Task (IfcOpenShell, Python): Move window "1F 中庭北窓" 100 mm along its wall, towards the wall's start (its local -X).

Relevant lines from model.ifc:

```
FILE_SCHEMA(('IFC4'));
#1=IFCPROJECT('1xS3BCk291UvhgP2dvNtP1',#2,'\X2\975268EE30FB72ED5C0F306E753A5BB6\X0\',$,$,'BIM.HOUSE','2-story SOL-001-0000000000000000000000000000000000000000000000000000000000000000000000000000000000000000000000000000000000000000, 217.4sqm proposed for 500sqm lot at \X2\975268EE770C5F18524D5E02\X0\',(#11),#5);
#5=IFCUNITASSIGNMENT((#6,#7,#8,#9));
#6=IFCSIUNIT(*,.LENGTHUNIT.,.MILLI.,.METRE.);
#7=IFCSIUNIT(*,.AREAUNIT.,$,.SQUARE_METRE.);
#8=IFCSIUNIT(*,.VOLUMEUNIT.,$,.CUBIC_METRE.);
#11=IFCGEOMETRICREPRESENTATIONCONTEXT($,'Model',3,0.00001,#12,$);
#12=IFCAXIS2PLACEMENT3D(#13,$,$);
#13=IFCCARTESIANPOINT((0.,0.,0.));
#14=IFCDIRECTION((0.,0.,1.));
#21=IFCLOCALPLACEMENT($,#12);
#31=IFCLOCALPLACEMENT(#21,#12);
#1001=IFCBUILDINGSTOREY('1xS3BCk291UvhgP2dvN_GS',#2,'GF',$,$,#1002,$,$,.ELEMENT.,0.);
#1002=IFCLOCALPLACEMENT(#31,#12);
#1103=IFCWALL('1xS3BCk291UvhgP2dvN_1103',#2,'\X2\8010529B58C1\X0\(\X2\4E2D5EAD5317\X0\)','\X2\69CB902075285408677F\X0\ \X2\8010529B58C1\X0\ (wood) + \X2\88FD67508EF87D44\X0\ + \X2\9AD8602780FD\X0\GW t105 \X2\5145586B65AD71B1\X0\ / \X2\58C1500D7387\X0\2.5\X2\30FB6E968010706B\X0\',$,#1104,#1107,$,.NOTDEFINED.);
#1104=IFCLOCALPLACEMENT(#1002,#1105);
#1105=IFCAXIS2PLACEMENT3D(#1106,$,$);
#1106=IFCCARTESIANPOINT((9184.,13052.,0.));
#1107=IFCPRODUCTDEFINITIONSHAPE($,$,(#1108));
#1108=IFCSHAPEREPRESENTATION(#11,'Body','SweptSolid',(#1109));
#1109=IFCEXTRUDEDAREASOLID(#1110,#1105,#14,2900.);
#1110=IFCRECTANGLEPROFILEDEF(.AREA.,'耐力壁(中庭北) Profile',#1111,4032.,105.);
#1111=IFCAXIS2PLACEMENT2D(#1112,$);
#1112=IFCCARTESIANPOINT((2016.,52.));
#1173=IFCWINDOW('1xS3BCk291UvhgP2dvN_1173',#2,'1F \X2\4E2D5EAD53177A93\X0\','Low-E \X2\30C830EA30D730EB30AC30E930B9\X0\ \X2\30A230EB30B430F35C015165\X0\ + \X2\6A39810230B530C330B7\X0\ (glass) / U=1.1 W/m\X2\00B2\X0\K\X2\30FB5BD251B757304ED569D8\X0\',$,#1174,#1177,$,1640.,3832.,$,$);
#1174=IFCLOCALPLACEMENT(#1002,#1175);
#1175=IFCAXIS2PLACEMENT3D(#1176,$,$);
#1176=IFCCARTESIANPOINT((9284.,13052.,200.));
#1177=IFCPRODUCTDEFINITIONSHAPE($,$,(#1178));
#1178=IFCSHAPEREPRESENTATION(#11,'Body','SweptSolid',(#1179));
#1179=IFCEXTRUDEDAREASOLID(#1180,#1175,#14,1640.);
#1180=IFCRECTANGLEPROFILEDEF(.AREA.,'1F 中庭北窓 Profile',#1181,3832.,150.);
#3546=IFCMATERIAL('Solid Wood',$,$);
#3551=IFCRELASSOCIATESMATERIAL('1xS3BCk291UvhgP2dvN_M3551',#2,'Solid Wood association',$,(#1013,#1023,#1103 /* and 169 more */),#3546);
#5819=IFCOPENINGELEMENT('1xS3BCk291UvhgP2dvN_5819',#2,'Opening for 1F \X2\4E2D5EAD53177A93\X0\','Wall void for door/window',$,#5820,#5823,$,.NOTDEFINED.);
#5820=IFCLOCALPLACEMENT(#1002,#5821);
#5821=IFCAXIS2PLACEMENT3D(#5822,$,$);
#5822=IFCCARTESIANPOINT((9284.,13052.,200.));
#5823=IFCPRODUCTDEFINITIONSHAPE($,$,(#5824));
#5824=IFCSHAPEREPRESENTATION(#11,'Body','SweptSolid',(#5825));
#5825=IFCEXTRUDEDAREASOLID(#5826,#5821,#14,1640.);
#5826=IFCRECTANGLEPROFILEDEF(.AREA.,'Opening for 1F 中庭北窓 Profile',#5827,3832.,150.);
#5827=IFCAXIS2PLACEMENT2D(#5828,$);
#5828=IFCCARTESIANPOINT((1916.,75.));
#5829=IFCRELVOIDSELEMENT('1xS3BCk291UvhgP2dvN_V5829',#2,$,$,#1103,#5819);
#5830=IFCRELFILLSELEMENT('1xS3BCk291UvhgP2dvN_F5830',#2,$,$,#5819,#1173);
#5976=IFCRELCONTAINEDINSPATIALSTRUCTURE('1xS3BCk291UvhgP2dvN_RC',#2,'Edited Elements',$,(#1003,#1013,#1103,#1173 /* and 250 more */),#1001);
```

```python
import ifcopenshell
import ifcopenshell.api.geometry
import ifcopenshell.util.placement

model = ifcopenshell.open("model.ifc")

window = model.by_guid("1xS3BCk291UvhgP2dvN_1173")
opening = window.FillsVoids[0].RelatingOpeningElement
wall = opening.VoidsElements[0].RelatingBuildingElement

wall_matrix = ifcopenshell.util.placement.get_local_placement(wall.ObjectPlacement)
shift = wall_matrix[:3, 0] * -100.0
before = ifcopenshell.util.placement.get_local_placement(window.ObjectPlacement)[:3, 3].copy()

# The window is not placed relative to its opening, so move both.
for product in (opening, window):
    matrix = ifcopenshell.util.placement.get_local_placement(product.ObjectPlacement)
    matrix[:3, 3] += shift
    ifcopenshell.api.geometry.edit_object_placement(model, product=product, matrix=matrix, is_si=False)

after = ifcopenshell.util.placement.get_local_placement(window.ObjectPlacement)[:3, 3]
print("window moved by", (after - before).round(3) + 0.0)

model.write("model_updated.ifc")
```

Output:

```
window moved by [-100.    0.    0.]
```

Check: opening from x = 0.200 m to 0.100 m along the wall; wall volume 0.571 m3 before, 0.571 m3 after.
